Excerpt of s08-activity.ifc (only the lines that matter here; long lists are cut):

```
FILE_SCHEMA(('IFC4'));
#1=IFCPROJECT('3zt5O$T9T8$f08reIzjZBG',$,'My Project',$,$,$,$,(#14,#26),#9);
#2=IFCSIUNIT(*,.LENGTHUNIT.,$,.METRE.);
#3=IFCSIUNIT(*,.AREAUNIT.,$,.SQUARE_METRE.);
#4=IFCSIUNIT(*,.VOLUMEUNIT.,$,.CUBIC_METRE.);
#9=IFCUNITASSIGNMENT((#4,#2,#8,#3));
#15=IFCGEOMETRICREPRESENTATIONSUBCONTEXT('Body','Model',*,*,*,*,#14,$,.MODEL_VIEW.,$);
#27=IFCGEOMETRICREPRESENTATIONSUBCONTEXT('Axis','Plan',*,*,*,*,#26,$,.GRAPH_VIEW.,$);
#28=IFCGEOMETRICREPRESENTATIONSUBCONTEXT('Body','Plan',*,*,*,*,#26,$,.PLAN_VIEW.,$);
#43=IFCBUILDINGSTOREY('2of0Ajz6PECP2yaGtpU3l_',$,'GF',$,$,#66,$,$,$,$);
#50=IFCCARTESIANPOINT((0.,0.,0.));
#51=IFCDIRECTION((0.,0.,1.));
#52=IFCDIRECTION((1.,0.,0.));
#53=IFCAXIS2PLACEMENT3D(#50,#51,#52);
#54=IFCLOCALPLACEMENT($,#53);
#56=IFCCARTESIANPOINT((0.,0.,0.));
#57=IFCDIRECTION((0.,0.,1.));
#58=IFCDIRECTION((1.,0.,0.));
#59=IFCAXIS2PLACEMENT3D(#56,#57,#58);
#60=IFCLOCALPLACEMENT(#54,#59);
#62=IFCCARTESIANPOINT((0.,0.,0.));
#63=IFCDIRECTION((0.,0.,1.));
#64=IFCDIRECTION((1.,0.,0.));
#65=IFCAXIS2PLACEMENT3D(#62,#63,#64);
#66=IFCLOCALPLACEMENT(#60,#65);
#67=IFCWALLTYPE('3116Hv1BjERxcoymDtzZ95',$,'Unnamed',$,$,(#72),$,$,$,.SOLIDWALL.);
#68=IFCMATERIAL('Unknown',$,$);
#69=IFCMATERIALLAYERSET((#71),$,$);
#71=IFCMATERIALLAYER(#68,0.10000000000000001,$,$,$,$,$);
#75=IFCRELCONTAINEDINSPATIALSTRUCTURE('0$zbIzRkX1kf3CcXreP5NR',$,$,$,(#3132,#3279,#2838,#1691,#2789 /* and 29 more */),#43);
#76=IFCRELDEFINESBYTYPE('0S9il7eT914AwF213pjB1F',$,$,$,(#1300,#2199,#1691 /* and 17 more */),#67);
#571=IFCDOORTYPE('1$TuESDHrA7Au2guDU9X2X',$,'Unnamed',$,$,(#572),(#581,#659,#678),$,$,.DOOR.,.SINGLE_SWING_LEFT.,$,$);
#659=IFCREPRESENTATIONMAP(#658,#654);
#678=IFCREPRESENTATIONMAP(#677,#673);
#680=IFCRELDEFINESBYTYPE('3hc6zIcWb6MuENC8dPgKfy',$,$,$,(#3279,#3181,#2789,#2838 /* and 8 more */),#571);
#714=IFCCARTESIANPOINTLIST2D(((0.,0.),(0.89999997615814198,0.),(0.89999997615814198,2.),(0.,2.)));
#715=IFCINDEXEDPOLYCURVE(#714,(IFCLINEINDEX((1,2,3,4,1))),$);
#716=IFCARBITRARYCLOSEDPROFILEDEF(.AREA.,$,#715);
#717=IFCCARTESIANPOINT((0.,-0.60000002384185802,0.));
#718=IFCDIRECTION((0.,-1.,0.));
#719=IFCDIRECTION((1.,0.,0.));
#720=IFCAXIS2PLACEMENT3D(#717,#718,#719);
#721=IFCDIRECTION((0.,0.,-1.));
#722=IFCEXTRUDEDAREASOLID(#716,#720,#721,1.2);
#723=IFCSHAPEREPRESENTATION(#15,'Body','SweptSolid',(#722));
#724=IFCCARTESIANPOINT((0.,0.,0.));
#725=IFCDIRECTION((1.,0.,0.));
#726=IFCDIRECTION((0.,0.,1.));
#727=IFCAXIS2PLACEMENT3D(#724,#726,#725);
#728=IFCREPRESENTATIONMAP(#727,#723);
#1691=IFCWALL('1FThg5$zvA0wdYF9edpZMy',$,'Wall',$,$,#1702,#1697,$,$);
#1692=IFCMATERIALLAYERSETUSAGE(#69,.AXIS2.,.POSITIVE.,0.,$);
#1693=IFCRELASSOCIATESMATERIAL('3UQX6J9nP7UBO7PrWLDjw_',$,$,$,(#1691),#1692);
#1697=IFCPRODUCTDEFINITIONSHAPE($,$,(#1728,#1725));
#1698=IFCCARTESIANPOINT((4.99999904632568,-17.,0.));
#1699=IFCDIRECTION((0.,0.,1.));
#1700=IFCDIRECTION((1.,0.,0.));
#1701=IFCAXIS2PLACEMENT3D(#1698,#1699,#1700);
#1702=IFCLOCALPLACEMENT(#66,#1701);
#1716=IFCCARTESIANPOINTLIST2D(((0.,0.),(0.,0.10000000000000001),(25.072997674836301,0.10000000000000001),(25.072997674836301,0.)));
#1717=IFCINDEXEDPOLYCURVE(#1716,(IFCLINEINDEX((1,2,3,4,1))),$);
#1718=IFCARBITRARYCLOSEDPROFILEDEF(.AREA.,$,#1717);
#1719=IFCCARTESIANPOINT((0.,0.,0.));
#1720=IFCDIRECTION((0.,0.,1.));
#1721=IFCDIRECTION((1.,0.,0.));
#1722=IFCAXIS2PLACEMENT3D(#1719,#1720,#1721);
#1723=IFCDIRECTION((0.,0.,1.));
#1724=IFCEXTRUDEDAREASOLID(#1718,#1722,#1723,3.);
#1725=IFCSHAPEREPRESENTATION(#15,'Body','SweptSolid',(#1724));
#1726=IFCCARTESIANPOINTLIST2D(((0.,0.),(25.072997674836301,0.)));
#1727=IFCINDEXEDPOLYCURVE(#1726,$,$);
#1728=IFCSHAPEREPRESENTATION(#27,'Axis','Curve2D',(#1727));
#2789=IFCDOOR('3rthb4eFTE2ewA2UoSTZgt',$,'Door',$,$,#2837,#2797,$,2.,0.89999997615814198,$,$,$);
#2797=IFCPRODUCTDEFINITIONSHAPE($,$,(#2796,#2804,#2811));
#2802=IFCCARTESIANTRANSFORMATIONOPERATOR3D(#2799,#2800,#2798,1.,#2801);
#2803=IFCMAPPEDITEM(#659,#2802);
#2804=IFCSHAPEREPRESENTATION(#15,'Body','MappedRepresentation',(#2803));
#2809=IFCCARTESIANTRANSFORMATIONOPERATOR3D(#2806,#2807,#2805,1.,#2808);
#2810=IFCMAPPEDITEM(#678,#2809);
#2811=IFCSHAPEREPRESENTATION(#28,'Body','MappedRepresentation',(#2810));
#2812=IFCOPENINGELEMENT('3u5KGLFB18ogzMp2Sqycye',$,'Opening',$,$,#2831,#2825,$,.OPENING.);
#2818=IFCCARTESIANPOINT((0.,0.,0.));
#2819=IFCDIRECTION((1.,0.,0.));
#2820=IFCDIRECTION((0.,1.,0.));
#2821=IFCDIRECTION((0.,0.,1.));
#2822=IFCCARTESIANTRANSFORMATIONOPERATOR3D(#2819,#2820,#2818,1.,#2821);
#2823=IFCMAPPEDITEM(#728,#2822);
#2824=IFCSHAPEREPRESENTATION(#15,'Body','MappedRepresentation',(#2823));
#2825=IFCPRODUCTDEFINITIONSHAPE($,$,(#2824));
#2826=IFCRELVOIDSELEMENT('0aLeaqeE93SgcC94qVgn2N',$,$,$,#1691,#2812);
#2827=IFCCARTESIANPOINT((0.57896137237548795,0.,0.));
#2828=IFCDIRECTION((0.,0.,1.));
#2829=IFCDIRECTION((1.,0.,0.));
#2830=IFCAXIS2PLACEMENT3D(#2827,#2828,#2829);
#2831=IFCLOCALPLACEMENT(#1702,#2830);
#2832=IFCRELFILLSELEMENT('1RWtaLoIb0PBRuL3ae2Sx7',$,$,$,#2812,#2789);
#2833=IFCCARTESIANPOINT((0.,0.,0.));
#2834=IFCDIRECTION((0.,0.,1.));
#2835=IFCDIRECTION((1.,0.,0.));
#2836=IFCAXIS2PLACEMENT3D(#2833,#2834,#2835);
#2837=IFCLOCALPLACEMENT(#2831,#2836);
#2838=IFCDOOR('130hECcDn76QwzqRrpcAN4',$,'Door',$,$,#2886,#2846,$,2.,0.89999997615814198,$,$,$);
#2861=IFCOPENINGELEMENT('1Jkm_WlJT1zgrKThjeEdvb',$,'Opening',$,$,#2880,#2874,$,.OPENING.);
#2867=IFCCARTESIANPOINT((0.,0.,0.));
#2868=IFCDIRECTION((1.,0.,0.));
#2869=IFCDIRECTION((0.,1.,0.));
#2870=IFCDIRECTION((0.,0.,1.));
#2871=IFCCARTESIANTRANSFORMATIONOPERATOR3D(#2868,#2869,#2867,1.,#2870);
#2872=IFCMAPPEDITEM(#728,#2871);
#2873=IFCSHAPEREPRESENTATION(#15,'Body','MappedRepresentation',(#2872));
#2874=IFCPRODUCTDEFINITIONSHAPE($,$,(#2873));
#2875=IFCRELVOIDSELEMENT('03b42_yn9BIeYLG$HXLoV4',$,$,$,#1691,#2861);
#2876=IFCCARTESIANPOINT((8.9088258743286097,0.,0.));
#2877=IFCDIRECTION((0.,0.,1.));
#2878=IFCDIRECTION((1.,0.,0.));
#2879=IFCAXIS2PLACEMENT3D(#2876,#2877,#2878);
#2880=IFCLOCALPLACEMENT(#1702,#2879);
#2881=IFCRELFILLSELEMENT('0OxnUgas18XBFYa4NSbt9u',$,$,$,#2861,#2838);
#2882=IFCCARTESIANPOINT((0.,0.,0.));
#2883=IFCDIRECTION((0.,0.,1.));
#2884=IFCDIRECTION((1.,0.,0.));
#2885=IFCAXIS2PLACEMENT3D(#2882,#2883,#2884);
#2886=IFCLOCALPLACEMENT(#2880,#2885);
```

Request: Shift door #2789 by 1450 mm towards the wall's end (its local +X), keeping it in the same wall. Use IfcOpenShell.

```python
import ifcopenshell
import ifcopenshell.api.geometry
import ifcopenshell.util.placement
import ifcopenshell.util.unit

model = ifcopenshell.open("s08-activity.ifc")
unit_scale = ifcopenshell.util.unit.calculate_unit_scale(model)

door = model.by_guid("3rthb4eFTE2ewA2UoSTZgt")
opening = door.FillsVoids[0].RelatingOpeningElement
wall = opening.VoidsElements[0].RelatingBuildingElement

wall_matrix = ifcopenshell.util.placement.get_local_placement(wall.ObjectPlacement)
shift = wall_matrix[:3, 0] * 1.45 / unit_scale
before = ifcopenshell.util.placement.get_local_placement(door.ObjectPlacement)[:3, 3].copy()

# The door is placed relative to its opening, so it follows when the opening moves.
matrix = ifcopenshell.util.placement.get_local_placement(opening.ObjectPlacement)
matrix[:3, 3] += shift
ifcopenshell.api.geometry.edit_object_placement(
    model, product=opening, matrix=matrix, is_si=False, should_transform_children=True
)

after = ifcopenshell.util.placement.get_local_placement(door.ObjectPlacement)[:3, 3]
print("door moved by", (after - before).round(3) + 0.0)

model.write("s08-activity_rev.ifc")
```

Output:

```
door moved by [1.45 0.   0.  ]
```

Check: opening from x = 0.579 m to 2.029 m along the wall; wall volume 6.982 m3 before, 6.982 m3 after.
